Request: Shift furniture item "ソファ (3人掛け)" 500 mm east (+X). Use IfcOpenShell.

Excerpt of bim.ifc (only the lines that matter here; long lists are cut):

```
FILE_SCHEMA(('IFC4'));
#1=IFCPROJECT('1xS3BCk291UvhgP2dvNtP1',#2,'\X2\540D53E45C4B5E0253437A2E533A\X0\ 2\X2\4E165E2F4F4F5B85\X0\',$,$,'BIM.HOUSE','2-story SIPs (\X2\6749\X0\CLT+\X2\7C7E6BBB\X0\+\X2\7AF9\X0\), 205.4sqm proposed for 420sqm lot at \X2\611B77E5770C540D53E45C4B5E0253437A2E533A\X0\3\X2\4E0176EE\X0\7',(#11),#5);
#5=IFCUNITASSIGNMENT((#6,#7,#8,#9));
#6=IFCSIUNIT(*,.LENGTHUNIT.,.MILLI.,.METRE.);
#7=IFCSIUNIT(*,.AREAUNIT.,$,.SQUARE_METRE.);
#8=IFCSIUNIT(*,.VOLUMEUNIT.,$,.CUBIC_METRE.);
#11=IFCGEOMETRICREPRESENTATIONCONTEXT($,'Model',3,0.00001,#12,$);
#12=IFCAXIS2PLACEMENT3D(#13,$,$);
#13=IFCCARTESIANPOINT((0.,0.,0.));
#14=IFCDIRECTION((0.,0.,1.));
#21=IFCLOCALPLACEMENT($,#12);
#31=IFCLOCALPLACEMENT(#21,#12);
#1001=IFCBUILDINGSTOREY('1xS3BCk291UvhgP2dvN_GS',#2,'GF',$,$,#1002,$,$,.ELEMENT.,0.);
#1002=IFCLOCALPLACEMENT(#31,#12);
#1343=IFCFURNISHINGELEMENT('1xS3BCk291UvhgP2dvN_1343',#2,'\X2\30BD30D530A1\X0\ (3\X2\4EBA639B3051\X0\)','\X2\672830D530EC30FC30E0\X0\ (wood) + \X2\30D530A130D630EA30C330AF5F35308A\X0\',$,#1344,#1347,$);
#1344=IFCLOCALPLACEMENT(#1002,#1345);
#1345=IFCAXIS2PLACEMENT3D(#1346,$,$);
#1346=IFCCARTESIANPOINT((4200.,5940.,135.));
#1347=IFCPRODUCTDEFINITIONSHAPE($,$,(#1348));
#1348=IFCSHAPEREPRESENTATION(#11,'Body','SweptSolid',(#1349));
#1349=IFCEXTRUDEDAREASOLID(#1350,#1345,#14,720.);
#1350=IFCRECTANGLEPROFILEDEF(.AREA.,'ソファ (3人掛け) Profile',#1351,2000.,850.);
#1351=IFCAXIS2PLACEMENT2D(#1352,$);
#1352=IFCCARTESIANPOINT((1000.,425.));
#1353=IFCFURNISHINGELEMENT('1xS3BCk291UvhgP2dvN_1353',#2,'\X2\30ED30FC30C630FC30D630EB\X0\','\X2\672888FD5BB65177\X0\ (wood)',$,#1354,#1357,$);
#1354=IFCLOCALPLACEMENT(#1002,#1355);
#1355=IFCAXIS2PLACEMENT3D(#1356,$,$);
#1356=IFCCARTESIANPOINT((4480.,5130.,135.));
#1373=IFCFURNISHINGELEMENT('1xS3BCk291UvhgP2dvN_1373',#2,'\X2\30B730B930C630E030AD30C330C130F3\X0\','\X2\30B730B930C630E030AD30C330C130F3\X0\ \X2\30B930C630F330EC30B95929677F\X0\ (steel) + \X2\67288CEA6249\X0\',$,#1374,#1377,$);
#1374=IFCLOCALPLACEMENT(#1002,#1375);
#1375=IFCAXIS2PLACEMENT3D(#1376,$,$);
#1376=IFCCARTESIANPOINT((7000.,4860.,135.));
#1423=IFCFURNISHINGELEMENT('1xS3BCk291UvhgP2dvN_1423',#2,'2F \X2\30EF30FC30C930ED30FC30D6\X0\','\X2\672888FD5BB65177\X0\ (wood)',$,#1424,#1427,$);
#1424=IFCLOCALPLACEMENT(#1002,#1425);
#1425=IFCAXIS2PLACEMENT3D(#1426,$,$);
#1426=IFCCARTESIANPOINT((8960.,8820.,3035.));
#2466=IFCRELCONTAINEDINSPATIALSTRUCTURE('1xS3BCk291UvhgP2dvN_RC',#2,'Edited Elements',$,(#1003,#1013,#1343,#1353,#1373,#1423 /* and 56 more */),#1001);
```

```python
import ifcopenshell
import ifcopenshell.api.geometry
import ifcopenshell.util.placement
import ifcopenshell.util.unit

model = ifcopenshell.open("bim.ifc")
unit_scale = ifcopenshell.util.unit.calculate_unit_scale(model)

item = model.by_guid("1xS3BCk291UvhgP2dvN_1343")
matrix = ifcopenshell.util.placement.get_local_placement(item.ObjectPlacement)
matrix[0, 3] += 0.5 / unit_scale
ifcopenshell.api.geometry.edit_object_placement(model, product=item, matrix=matrix, is_si=False)

print(ifcopenshell.util.placement.get_local_placement(item.ObjectPlacement).round(3) + 0.0)

model.write("bim_rev.ifc")
```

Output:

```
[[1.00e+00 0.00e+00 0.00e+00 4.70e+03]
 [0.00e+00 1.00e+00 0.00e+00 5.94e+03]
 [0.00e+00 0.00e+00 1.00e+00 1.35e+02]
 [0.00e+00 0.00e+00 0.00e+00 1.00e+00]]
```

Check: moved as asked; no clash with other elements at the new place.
